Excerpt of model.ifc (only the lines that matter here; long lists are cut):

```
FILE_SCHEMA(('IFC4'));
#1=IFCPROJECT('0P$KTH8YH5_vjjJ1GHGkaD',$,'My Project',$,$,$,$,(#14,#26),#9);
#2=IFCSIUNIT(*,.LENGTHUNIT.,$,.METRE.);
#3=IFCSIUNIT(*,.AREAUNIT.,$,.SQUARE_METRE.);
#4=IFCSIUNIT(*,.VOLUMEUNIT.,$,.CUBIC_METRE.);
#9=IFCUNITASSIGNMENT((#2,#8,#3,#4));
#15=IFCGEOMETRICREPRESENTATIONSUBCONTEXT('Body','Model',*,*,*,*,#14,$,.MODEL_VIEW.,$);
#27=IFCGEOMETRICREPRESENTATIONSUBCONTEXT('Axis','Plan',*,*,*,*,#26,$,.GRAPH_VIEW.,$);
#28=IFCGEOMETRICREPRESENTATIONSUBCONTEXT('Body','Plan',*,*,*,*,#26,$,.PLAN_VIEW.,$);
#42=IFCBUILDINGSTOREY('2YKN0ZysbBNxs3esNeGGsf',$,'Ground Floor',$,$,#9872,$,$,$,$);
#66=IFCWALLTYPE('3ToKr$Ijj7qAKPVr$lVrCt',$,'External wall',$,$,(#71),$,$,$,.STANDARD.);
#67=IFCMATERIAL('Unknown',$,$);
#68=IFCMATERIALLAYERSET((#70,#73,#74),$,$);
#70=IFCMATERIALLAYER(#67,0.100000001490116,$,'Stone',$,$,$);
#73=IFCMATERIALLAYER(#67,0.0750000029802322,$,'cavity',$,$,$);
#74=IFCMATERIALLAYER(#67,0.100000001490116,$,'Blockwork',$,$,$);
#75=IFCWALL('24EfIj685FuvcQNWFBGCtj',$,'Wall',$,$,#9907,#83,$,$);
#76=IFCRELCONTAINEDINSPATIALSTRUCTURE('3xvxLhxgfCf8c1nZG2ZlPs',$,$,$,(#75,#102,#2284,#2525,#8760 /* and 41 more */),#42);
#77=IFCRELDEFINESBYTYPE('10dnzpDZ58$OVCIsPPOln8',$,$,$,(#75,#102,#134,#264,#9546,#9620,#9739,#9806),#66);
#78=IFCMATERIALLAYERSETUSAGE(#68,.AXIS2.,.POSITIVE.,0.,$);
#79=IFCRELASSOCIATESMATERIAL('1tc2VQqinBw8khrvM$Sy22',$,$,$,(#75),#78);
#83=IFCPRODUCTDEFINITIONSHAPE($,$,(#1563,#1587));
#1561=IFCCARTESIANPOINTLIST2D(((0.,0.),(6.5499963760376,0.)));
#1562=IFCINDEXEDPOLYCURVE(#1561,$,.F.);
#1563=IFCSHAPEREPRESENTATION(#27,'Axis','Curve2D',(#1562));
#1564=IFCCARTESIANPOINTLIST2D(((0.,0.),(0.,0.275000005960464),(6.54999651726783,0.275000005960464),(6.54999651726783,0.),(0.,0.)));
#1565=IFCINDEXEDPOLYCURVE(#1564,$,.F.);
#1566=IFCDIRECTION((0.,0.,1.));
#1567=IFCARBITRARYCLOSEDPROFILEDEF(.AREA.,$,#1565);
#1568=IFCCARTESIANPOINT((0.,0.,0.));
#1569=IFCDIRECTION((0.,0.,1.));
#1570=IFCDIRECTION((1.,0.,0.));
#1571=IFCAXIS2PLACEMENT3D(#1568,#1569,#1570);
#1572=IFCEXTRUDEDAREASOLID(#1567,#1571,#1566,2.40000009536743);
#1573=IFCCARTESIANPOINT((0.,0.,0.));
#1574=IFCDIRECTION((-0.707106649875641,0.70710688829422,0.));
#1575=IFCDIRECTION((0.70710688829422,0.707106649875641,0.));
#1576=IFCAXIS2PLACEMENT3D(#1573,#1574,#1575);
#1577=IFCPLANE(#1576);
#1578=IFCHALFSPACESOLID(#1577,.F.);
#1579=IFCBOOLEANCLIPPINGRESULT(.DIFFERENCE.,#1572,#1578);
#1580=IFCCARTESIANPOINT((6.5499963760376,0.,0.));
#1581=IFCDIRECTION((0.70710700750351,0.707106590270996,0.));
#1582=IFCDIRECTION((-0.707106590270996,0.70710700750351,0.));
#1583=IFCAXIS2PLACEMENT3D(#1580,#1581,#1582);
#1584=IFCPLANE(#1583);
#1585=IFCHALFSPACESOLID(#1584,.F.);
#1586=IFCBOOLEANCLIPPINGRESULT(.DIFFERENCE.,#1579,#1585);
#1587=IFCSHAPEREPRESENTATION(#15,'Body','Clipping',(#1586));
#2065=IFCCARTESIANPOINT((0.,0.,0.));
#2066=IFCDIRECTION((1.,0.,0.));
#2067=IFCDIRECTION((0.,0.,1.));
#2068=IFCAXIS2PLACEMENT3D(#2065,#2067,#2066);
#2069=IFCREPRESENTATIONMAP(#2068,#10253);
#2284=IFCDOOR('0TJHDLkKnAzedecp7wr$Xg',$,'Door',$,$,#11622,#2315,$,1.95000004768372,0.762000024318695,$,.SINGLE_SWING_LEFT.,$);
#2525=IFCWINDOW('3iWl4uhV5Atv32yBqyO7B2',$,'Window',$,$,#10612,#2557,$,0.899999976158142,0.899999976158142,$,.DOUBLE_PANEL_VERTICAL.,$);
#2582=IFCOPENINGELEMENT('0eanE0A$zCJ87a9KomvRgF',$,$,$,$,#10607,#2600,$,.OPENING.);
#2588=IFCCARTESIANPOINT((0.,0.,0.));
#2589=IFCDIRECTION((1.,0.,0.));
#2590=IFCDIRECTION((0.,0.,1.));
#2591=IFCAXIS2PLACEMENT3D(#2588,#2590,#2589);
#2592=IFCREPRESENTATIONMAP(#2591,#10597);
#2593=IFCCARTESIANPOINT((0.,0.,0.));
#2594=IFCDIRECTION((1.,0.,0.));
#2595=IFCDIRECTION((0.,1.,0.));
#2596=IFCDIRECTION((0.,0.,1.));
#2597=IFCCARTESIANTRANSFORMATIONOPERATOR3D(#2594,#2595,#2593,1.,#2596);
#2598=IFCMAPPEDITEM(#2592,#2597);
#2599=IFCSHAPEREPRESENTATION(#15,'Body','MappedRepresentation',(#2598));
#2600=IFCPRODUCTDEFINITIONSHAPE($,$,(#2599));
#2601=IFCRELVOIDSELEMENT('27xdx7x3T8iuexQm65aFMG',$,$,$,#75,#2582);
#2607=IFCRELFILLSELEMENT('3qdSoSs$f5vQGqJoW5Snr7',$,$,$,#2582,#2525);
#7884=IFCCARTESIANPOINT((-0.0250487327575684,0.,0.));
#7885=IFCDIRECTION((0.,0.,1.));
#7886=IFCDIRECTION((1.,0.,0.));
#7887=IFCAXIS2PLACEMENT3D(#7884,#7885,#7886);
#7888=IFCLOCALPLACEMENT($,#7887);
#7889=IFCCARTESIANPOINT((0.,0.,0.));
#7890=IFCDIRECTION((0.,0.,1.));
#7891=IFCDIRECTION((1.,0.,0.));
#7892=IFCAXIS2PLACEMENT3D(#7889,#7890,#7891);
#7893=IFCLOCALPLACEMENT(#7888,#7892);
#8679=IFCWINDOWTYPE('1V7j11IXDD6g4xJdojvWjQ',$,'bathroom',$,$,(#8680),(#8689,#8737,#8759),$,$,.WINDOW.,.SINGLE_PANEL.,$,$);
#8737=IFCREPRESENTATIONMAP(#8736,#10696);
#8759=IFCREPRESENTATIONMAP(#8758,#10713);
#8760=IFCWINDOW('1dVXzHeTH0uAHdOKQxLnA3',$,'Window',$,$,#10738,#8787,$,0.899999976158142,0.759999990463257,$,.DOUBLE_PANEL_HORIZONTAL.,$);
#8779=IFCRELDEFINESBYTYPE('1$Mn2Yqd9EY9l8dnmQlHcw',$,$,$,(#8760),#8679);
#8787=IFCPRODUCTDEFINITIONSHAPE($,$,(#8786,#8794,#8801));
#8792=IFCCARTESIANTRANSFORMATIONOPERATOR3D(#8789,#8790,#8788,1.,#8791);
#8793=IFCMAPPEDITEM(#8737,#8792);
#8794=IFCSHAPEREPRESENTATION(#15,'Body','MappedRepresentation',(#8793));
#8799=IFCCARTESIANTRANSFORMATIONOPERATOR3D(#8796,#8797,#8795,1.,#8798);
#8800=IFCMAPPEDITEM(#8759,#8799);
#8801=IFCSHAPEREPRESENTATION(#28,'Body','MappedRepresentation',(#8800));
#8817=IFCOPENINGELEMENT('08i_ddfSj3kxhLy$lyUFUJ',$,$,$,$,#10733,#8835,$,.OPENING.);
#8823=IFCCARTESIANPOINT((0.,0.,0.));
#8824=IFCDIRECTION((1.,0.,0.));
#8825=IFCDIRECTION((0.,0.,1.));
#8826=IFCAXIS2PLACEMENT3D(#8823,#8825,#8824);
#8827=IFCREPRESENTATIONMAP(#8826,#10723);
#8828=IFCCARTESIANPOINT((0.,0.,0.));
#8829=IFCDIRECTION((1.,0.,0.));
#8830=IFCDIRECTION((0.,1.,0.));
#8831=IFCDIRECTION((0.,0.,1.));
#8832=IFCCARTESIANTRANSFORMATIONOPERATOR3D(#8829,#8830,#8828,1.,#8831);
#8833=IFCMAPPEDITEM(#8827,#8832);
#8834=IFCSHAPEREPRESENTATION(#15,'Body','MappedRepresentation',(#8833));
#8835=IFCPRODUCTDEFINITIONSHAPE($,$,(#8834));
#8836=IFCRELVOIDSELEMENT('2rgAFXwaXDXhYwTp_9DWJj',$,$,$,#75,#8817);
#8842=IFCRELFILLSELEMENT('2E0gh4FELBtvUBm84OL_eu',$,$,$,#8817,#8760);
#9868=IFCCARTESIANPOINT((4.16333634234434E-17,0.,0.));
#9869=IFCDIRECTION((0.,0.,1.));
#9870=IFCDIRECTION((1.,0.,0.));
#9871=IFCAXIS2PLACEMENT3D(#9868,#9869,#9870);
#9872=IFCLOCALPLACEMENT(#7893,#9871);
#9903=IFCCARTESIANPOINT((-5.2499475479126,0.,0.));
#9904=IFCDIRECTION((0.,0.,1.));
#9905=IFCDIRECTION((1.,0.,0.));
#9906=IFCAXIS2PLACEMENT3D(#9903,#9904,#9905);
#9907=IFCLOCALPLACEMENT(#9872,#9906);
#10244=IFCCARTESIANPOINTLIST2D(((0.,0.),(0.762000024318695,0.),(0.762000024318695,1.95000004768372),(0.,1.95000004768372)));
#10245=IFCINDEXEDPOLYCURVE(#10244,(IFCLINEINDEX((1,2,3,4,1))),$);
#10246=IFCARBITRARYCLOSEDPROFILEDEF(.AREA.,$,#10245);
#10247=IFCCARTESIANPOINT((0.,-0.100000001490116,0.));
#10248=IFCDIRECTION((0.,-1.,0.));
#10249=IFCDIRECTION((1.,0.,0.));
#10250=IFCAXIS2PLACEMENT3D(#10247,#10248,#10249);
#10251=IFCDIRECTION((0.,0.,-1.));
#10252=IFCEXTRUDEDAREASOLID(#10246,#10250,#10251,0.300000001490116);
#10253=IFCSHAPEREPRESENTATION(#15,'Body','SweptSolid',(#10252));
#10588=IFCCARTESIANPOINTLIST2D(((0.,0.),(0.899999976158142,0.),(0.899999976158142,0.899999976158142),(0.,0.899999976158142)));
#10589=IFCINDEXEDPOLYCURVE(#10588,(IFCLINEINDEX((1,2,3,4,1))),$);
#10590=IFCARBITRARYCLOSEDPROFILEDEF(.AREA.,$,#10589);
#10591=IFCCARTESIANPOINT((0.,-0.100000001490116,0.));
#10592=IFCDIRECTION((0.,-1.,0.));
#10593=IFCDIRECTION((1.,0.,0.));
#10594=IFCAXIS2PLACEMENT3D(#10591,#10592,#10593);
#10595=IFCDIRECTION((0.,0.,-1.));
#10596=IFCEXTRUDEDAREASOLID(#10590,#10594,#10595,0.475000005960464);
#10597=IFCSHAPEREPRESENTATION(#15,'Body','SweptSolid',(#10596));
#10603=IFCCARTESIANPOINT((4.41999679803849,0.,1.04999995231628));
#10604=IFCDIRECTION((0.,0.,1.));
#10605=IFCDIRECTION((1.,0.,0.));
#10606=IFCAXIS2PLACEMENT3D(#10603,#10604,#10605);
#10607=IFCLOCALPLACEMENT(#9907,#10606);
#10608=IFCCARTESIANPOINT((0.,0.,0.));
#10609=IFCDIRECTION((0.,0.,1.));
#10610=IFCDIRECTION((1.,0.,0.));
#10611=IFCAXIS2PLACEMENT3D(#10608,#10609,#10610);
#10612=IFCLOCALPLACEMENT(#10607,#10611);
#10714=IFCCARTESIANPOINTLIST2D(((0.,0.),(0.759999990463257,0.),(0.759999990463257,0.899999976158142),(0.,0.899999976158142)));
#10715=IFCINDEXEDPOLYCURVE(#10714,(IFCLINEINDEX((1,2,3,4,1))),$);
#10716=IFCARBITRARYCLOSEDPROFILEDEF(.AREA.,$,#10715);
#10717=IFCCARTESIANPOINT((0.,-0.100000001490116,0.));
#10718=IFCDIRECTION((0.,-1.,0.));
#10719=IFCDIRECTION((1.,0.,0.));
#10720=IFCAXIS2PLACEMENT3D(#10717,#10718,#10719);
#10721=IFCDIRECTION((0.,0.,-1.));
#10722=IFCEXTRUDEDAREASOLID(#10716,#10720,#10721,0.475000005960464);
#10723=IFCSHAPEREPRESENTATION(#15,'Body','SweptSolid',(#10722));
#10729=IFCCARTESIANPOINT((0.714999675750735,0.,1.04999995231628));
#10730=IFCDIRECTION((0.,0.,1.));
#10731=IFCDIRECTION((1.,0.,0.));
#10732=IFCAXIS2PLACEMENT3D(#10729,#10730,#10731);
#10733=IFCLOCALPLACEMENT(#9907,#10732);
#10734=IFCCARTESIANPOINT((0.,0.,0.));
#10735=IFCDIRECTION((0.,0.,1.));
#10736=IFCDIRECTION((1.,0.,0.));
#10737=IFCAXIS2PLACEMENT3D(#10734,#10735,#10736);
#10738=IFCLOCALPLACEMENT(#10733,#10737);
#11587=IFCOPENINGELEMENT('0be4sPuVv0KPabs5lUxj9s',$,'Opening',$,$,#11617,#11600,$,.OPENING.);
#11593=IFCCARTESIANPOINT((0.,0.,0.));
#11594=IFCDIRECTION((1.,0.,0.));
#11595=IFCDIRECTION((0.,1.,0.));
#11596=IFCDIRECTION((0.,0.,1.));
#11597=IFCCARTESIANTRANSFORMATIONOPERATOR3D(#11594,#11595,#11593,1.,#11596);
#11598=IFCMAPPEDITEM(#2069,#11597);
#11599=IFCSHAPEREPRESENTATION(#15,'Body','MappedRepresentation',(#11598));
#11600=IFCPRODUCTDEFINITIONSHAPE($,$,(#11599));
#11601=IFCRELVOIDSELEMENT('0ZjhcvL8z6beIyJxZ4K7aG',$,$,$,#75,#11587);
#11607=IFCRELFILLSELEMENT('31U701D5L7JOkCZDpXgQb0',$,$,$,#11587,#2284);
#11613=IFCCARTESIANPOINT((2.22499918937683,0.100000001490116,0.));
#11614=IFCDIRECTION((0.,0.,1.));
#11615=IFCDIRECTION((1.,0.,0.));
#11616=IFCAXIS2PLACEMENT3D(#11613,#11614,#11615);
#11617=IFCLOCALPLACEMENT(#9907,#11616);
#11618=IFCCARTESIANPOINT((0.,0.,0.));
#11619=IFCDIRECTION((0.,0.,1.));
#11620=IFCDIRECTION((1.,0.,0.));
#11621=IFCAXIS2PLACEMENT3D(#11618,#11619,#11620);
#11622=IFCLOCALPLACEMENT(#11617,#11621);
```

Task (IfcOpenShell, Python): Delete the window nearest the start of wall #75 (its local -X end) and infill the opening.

```python
import ifcopenshell
import ifcopenshell.api.feature
import ifcopenshell.api.root
import ifcopenshell.geom
import ifcopenshell.util.shape

model = ifcopenshell.open("model.ifc")
settings = ifcopenshell.geom.settings()


def volume(element):
    """Net volume in cubic metres, openings subtracted."""
    shape = ifcopenshell.geom.create_shape(settings, element)
    return ifcopenshell.util.shape.get_volume(shape.geometry)


window = model.by_guid("1dVXzHeTH0uAHdOKQxLnA3")
opening = window.FillsVoids[0].RelatingOpeningElement
wall = opening.VoidsElements[0].RelatingBuildingElement
before = volume(wall)

ifcopenshell.api.root.remove_product(model, product=window)
ifcopenshell.api.feature.remove_feature(model, feature=opening)

after = volume(wall)

print(f"wall volume {before:.3f} -> {after:.3f} m3")

model.write("model-out.ifc")
```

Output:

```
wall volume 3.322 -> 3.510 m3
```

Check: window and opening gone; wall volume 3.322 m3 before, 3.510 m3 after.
